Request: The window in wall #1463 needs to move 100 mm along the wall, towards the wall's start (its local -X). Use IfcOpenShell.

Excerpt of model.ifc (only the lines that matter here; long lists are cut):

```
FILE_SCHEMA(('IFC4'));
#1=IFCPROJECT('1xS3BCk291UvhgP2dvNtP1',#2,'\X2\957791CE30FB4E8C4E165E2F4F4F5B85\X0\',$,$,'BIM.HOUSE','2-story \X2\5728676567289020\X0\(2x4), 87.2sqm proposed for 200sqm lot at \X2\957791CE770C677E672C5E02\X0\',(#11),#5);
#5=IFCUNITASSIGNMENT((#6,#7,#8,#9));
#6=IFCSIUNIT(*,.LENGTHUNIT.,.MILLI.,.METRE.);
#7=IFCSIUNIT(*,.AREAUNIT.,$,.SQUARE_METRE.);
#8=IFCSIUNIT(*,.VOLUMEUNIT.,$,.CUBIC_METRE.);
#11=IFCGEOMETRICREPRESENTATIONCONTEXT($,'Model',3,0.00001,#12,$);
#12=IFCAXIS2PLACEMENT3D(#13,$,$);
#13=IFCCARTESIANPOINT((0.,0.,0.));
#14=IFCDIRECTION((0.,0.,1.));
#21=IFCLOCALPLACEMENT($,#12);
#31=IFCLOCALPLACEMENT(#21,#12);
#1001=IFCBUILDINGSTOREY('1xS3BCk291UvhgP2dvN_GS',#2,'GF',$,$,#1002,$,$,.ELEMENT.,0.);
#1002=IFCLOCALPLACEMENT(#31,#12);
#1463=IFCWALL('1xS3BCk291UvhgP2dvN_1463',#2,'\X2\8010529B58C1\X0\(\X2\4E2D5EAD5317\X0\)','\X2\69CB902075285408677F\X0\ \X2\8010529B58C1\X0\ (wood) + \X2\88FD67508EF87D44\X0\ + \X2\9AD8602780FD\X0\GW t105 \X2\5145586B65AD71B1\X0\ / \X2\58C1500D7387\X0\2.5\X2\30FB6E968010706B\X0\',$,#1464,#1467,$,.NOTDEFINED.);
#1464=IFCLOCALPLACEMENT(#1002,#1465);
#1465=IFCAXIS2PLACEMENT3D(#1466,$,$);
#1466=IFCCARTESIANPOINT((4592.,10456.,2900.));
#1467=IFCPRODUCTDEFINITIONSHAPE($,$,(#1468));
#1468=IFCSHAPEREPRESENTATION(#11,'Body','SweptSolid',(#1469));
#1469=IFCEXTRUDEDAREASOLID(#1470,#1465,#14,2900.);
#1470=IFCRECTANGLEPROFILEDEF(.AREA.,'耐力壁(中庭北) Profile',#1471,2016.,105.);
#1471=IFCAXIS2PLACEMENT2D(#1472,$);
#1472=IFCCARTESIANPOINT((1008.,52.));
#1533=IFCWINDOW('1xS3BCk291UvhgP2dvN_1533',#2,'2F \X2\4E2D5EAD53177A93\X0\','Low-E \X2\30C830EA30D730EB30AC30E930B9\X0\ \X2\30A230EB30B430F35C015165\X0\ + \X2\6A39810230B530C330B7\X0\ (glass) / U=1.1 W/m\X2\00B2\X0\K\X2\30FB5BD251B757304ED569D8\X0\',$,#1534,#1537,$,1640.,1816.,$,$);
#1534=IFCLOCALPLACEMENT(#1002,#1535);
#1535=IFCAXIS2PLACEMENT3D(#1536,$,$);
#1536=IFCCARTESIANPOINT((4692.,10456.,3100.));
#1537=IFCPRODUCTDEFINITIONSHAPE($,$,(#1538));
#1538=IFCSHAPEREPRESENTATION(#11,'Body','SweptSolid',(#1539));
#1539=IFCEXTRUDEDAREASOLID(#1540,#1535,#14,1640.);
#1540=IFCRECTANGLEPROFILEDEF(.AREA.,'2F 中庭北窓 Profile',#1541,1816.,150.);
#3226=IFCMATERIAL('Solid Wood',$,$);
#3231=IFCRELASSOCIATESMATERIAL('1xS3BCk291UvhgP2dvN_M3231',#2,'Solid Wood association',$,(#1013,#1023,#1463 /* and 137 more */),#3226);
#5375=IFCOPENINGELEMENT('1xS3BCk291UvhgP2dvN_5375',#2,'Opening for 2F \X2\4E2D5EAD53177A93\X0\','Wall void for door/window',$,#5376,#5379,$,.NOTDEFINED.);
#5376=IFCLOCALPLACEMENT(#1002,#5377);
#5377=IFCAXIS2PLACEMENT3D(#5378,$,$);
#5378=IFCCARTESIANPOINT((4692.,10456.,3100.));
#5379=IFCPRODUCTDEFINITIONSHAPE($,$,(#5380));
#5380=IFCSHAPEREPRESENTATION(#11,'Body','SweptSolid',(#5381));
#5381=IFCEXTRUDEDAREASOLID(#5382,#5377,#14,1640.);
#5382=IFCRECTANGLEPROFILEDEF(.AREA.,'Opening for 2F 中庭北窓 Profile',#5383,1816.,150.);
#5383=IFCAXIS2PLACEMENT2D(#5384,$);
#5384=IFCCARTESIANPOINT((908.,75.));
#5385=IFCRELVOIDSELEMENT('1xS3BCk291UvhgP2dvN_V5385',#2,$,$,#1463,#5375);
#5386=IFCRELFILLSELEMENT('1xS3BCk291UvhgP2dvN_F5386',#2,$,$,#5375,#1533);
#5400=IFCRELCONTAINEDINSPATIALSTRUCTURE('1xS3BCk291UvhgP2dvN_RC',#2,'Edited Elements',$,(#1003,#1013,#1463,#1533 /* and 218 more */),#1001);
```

```python
import ifcopenshell
import ifcopenshell.api.geometry
import ifcopenshell.util.placement
import ifcopenshell.util.unit

model = ifcopenshell.open("model.ifc")
unit_scale = ifcopenshell.util.unit.calculate_unit_scale(model)

window = model.by_id(1533)
opening = window.FillsVoids[0].RelatingOpeningElement
wall = opening.VoidsElements[0].RelatingBuildingElement

wall_matrix = ifcopenshell.util.placement.get_local_placement(wall.ObjectPlacement)
shift = wall_matrix[:3, 0] * -0.1 / unit_scale
before = ifcopenshell.util.placement.get_local_placement(window.ObjectPlacement)[:3, 3].copy()

# The window is not placed relative to its opening, so move both.
for product in (opening, window):
    matrix = ifcopenshell.util.placement.get_local_placement(product.ObjectPlacement)
    matrix[:3, 3] += shift
    ifcopenshell.api.geometry.edit_object_placement(model, product=product, matrix=matrix, is_si=False)

after = ifcopenshell.util.placement.get_local_placement(window.ObjectPlacement)[:3, 3]
print("window moved by", (after - before).round(3) + 0.0)

model.write("model_v2.ifc")
```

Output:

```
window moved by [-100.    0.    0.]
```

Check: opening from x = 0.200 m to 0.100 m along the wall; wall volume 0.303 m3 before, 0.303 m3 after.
